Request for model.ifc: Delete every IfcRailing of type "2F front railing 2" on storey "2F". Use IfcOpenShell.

First a look at what the model holds.

```python
import ifcopenshell
import ifcopenshell.util.element

model = ifcopenshell.open("model.ifc")
print(model.schema)
storey = next(s for s in model.by_type("IfcBuildingStorey") if s.Name == "2F")
railings = [e for e in ifcopenshell.util.element.get_decomposition(storey) if e.is_a("IfcRailing")]
seen = {}
for e in railings:
    element_type = ifcopenshell.util.element.get_type(e)
    name = element_type.Name if element_type not in (None, e) else None
    seen[name] = seen.get(name, 0) + 1
for name, count in sorted(seen.items(), key=str):
    print(count, "x", name)
```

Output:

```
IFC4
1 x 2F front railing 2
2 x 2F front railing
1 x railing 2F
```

```python
import ifcopenshell
import ifcopenshell.api.root
import ifcopenshell.util.element

model = ifcopenshell.open("model.ifc")

storey = next(s for s in model.by_type("IfcBuildingStorey") if s.Name == "2F")
railings = [e for e in ifcopenshell.util.element.get_decomposition(storey) if e.is_a("IfcRailing")]
targets = [e for e in railings if (t := ifcopenshell.util.element.get_type(e)) not in (None, e) and t.Name == "2F front railing 2"]

for e in targets:
    ifcopenshell.api.root.remove_product(model, product=e)
print(len(targets), "removed")

model.write("model-out.ifc")
```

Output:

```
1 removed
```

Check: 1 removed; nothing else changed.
